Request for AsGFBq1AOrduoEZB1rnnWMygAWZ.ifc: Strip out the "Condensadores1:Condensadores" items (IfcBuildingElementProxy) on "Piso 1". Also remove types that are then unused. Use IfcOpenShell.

First a look at what the model holds.

```python
import ifcopenshell
import ifcopenshell.util.element

model = ifcopenshell.open("AsGFBq1AOrduoEZB1rnnWMygAWZ.ifc")
print(model.schema)
storey = next(s for s in model.by_type("IfcBuildingStorey") if s.Name == "Piso 1")
proxies = [e for e in ifcopenshell.util.element.get_decomposition(storey) if e.is_a("IfcBuildingElementProxy")]
seen = {}
for e in proxies:
    element_type = ifcopenshell.util.element.get_type(e)
    name = element_type.Name if element_type not in (None, e) else None
    seen[name] = seen.get(name, 0) + 1
for name, count in sorted(seen.items(), key=str):
    print(count, "x", name)
```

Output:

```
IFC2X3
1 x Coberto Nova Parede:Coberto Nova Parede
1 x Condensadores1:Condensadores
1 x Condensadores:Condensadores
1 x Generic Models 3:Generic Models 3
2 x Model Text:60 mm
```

```python
import ifcopenshell
import ifcopenshell.api.root
import ifcopenshell.util.element

model = ifcopenshell.open("AsGFBq1AOrduoEZB1rnnWMygAWZ.ifc")

storey = next(s for s in model.by_type("IfcBuildingStorey") if s.Name == "Piso 1")
proxies = [e for e in ifcopenshell.util.element.get_decomposition(storey) if e.is_a("IfcBuildingElementProxy")]
targets = [e for e in proxies if (t := ifcopenshell.util.element.get_type(e)) not in (None, e) and t.Name == "Condensadores1:Condensadores"]
types = {ifcopenshell.util.element.get_type(e) for e in targets} - {None, *targets}

for e in targets:
    ifcopenshell.api.root.remove_product(model, product=e)
print(len(targets), "removed")

unused = [t for t in types if not ifcopenshell.util.element.get_types(t)]
for t in unused:
    ifcopenshell.api.root.remove_product(model, product=t)
print(len(unused), "unused types removed")

model.write("AsGFBq1AOrduoEZB1rnnWMygAWZ_edited.ifc")
```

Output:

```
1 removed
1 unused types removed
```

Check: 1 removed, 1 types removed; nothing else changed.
